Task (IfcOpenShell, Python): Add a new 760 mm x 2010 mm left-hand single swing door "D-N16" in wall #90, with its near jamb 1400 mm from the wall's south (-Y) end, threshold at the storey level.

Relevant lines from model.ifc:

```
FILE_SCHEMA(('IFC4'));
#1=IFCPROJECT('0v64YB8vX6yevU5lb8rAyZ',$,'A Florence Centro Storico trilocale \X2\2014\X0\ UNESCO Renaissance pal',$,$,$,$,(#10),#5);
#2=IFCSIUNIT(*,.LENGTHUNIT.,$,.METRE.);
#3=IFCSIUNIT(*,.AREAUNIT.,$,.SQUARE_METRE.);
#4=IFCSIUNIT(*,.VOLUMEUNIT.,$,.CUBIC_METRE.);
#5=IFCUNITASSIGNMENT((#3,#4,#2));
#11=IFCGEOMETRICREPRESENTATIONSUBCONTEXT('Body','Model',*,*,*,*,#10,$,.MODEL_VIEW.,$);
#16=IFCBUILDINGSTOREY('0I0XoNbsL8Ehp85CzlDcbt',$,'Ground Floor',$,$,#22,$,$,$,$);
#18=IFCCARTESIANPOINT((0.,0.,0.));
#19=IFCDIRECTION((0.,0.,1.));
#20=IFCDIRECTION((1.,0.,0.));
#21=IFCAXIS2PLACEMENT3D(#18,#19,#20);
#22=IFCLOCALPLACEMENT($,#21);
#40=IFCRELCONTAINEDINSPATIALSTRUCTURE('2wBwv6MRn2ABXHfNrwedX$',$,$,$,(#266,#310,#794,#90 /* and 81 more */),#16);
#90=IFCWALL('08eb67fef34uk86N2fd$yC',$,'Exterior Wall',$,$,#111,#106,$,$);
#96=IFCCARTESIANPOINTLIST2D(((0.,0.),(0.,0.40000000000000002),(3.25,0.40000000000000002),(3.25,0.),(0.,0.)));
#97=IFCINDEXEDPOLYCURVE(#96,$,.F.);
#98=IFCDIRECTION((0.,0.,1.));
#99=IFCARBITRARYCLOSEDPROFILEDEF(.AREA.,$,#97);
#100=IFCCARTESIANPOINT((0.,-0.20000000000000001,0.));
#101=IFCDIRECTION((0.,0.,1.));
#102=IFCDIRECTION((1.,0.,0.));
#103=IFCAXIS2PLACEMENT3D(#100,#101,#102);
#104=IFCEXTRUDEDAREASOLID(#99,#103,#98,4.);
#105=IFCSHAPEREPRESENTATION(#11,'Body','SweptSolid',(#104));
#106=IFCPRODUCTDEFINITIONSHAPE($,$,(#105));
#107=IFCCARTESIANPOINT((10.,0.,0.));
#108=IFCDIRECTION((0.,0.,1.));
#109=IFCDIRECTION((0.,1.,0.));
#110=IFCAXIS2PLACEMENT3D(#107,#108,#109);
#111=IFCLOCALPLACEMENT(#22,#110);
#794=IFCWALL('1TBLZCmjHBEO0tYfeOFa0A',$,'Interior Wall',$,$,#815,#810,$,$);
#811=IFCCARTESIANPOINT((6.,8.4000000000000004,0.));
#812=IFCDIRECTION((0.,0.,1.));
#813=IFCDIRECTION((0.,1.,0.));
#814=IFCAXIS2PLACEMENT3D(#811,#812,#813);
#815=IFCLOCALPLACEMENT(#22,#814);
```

```python
import numpy as np
import ifcopenshell
import ifcopenshell.api.feature
import ifcopenshell.api.geometry
import ifcopenshell.api.root
import ifcopenshell.api.spatial
import ifcopenshell.geom
import ifcopenshell.util.element
import ifcopenshell.util.placement
import ifcopenshell.util.representation
import ifcopenshell.util.shape
import ifcopenshell.util.unit

model = ifcopenshell.open("model.ifc")
unit_scale = ifcopenshell.util.unit.calculate_unit_scale(model)
settings = ifcopenshell.geom.settings()


def volume(element):
    """Net volume in cubic metres, openings subtracted."""
    shape = ifcopenshell.geom.create_shape(settings, element)
    return ifcopenshell.util.shape.get_volume(shape.geometry)


wall = model.by_guid("08eb67fef34uk86N2fd$yC")
storey = ifcopenshell.util.element.get_container(wall, ifc_class="IfcBuildingStorey")
context = ifcopenshell.util.representation.get_context(model, "Model", "Body", "MODEL_VIEW")
before = volume(wall)

width, height, from_end, sill = 0.76, 2.01, 1.4, 0.0  # metres

# The wall runs along its own X axis, and the end named is its -X end.
wall_shape = ifcopenshell.geom.create_shape(settings, wall)
x, y, z = ifcopenshell.util.shape.get_vertices(wall_shape.geometry).T
start = x.min() + from_end
face, thickness = float(y.min()), float(y.max() - y.min())
wall_matrix = ifcopenshell.util.placement.get_local_placement(wall.ObjectPlacement)
level = ifcopenshell.util.placement.get_local_placement(storey.ObjectPlacement)[2, 3]


def in_wall(x, y):
    """Placement at x, y metres in the wall's axes, at sill height."""
    matrix = wall_matrix.copy()
    matrix[:, 3] = wall_matrix @ np.array([x / unit_scale, y / unit_scale, 0.0, 1.0])
    matrix[2, 3] = level + sill / unit_scale
    return matrix


# Opening: a box that overshoots both wall faces by 50 mm.
opening = ifcopenshell.api.root.create_entity(model, ifc_class="IfcOpeningElement", predefined_type="OPENING")
box = ifcopenshell.api.geometry.add_wall_representation(
    model, context=context, length=width, height=height, thickness=thickness + 0.1
)
ifcopenshell.api.geometry.assign_representation(model, product=opening, representation=box)
ifcopenshell.api.geometry.edit_object_placement(model, product=opening, matrix=in_wall(start, face - 0.05), is_si=False)
ifcopenshell.api.feature.add_feature(model, feature=opening, element=wall)

door = ifcopenshell.api.root.create_entity(model, ifc_class="IfcDoor", name="D-N16", predefined_type="DOOR")
door.OverallWidth, door.OverallHeight = width / unit_scale, height / unit_scale
door.OperationType = "SINGLE_SWING_LEFT"
body = ifcopenshell.api.geometry.add_door_representation(
    model,
    context=context,
    overall_width=door.OverallWidth,
    overall_height=door.OverallHeight,
    operation_type="SINGLE_SWING_LEFT",
    lining_properties={"LiningDepth": thickness / unit_scale, "ThresholdDepth": thickness / unit_scale},
)
ifcopenshell.api.geometry.assign_representation(model, product=door, representation=body)
ifcopenshell.api.spatial.assign_container(model, products=[door], relating_structure=storey)
ifcopenshell.api.feature.add_filling(model, opening=opening, element=door)

# The lining spans the wall, so the door starts at the wall face.
ifcopenshell.api.geometry.edit_object_placement(model, product=door, matrix=in_wall(start, face), is_si=False)

after = volume(wall)

print(f"wall volume {before:.3f} -> {after:.3f} m3")

model.write("model_rev.ifc")
```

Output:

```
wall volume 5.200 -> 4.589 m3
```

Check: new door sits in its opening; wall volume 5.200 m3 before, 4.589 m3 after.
